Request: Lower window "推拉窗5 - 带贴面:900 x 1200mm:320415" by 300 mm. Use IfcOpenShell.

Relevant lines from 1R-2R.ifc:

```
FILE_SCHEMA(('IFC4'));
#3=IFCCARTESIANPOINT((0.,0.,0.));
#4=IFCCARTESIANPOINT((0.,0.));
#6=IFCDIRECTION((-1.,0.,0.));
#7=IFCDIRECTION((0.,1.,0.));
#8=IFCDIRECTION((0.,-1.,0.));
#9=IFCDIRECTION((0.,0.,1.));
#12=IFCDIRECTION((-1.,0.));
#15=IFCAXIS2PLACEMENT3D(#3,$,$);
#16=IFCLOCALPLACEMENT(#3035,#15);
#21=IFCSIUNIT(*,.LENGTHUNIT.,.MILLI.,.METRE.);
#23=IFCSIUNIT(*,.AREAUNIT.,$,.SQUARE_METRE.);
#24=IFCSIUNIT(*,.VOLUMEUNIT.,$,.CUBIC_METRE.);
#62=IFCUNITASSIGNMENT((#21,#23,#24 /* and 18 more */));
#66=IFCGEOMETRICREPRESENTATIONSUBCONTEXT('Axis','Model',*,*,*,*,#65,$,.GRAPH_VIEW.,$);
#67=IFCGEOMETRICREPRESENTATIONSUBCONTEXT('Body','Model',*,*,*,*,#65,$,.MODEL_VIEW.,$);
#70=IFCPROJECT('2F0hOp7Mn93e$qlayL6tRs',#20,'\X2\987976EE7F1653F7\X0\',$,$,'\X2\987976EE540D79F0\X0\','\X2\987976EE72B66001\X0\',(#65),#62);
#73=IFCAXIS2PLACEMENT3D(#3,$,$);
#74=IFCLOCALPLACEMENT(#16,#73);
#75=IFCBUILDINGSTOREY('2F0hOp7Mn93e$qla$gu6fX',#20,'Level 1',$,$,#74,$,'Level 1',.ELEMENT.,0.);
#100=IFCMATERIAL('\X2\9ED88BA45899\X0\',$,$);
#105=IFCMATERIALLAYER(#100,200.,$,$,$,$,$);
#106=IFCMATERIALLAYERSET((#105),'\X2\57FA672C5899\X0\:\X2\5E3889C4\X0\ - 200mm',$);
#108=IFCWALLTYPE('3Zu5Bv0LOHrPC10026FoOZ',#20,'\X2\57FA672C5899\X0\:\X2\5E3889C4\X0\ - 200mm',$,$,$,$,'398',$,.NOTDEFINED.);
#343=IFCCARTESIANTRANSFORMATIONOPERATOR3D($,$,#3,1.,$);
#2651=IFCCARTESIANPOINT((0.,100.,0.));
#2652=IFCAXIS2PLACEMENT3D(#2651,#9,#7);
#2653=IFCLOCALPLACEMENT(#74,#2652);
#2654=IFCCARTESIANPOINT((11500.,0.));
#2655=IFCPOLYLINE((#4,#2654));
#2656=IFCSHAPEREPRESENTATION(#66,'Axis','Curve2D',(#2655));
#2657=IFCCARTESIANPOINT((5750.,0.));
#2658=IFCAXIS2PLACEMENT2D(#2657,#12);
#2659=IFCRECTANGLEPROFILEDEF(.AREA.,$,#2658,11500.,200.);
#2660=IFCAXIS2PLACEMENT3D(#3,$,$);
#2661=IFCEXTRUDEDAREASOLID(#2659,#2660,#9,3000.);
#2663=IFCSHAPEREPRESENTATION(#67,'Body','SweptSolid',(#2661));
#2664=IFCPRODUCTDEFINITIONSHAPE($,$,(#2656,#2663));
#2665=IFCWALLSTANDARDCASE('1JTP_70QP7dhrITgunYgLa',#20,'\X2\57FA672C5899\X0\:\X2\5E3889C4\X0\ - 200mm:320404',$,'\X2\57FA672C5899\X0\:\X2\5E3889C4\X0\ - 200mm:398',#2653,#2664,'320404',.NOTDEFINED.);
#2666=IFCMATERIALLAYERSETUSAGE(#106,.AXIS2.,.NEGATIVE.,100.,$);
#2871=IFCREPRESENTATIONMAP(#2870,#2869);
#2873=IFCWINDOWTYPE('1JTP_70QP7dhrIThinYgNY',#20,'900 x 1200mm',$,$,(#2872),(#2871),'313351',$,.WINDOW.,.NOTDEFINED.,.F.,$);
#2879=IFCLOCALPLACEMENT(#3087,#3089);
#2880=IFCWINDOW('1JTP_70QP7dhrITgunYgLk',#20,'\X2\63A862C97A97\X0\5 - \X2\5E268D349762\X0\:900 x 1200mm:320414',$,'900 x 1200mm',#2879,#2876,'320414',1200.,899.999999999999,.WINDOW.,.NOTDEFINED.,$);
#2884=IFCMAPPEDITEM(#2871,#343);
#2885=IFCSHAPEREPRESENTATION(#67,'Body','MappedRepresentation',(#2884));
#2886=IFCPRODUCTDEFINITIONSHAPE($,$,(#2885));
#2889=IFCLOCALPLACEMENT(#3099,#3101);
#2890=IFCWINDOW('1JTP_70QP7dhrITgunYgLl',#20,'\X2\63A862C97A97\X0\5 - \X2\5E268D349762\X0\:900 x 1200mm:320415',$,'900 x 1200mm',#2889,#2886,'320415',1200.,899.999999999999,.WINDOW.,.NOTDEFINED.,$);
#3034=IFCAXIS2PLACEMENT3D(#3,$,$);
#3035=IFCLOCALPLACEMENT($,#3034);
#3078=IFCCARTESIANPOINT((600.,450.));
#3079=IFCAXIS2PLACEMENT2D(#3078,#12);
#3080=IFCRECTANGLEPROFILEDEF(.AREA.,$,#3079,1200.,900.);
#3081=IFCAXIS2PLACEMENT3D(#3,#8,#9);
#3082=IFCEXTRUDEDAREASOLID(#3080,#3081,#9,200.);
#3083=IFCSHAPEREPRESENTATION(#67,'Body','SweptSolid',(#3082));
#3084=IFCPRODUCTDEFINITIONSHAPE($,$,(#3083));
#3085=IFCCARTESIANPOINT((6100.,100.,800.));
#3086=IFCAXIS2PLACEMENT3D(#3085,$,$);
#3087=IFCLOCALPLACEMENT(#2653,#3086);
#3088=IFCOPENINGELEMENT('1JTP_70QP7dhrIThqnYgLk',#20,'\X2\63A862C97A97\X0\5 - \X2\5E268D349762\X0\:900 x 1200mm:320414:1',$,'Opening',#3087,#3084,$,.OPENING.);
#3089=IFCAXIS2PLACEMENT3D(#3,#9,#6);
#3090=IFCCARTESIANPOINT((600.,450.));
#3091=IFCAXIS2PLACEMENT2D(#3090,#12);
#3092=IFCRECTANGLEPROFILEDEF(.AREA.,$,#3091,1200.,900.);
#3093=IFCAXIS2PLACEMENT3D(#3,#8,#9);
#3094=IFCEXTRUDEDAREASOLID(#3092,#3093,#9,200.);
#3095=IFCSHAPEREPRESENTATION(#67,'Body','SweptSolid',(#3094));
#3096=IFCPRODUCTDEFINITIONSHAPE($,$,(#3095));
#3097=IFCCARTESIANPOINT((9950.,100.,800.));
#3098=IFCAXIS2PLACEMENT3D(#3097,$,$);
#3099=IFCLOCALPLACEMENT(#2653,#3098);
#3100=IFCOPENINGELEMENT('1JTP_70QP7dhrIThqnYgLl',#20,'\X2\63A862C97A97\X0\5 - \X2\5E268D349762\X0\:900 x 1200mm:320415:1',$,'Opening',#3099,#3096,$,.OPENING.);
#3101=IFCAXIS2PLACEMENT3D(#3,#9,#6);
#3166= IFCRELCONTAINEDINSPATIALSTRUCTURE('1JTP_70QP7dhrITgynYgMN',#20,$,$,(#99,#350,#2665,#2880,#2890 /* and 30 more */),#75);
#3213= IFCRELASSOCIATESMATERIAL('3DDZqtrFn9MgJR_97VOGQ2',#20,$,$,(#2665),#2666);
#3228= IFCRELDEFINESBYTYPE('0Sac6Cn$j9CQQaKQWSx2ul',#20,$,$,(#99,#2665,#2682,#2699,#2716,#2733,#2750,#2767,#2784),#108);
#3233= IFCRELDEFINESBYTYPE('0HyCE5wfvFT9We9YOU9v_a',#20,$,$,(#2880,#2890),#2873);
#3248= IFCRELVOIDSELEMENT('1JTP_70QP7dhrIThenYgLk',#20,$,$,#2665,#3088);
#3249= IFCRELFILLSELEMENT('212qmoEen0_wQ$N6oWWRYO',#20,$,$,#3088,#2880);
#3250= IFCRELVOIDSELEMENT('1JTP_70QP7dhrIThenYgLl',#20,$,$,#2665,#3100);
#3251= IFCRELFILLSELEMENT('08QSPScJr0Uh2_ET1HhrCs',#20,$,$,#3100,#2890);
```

```python
import numpy as np
import ifcopenshell
import ifcopenshell.api.geometry
import ifcopenshell.util.placement
import ifcopenshell.util.unit

model = ifcopenshell.open("1R-2R.ifc")
unit_scale = ifcopenshell.util.unit.calculate_unit_scale(model)

window = model.by_guid("1JTP_70QP7dhrITgunYgLl")
opening = window.FillsVoids[0].RelatingOpeningElement
dz = -300.0

shift = np.array([0.0, 0.0, dz])
# The window is placed relative to its opening, so it follows when the opening moves.
matrix = ifcopenshell.util.placement.get_local_placement(opening.ObjectPlacement)
matrix[:3, 3] += shift
ifcopenshell.api.geometry.edit_object_placement(
    model, product=opening, matrix=matrix, is_si=False, should_transform_children=True
)

print(f"moved by {dz * unit_scale:+.3f} m")

model.write("1R-2R-out.ifc")
```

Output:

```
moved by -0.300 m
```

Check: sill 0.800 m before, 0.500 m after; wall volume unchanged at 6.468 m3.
